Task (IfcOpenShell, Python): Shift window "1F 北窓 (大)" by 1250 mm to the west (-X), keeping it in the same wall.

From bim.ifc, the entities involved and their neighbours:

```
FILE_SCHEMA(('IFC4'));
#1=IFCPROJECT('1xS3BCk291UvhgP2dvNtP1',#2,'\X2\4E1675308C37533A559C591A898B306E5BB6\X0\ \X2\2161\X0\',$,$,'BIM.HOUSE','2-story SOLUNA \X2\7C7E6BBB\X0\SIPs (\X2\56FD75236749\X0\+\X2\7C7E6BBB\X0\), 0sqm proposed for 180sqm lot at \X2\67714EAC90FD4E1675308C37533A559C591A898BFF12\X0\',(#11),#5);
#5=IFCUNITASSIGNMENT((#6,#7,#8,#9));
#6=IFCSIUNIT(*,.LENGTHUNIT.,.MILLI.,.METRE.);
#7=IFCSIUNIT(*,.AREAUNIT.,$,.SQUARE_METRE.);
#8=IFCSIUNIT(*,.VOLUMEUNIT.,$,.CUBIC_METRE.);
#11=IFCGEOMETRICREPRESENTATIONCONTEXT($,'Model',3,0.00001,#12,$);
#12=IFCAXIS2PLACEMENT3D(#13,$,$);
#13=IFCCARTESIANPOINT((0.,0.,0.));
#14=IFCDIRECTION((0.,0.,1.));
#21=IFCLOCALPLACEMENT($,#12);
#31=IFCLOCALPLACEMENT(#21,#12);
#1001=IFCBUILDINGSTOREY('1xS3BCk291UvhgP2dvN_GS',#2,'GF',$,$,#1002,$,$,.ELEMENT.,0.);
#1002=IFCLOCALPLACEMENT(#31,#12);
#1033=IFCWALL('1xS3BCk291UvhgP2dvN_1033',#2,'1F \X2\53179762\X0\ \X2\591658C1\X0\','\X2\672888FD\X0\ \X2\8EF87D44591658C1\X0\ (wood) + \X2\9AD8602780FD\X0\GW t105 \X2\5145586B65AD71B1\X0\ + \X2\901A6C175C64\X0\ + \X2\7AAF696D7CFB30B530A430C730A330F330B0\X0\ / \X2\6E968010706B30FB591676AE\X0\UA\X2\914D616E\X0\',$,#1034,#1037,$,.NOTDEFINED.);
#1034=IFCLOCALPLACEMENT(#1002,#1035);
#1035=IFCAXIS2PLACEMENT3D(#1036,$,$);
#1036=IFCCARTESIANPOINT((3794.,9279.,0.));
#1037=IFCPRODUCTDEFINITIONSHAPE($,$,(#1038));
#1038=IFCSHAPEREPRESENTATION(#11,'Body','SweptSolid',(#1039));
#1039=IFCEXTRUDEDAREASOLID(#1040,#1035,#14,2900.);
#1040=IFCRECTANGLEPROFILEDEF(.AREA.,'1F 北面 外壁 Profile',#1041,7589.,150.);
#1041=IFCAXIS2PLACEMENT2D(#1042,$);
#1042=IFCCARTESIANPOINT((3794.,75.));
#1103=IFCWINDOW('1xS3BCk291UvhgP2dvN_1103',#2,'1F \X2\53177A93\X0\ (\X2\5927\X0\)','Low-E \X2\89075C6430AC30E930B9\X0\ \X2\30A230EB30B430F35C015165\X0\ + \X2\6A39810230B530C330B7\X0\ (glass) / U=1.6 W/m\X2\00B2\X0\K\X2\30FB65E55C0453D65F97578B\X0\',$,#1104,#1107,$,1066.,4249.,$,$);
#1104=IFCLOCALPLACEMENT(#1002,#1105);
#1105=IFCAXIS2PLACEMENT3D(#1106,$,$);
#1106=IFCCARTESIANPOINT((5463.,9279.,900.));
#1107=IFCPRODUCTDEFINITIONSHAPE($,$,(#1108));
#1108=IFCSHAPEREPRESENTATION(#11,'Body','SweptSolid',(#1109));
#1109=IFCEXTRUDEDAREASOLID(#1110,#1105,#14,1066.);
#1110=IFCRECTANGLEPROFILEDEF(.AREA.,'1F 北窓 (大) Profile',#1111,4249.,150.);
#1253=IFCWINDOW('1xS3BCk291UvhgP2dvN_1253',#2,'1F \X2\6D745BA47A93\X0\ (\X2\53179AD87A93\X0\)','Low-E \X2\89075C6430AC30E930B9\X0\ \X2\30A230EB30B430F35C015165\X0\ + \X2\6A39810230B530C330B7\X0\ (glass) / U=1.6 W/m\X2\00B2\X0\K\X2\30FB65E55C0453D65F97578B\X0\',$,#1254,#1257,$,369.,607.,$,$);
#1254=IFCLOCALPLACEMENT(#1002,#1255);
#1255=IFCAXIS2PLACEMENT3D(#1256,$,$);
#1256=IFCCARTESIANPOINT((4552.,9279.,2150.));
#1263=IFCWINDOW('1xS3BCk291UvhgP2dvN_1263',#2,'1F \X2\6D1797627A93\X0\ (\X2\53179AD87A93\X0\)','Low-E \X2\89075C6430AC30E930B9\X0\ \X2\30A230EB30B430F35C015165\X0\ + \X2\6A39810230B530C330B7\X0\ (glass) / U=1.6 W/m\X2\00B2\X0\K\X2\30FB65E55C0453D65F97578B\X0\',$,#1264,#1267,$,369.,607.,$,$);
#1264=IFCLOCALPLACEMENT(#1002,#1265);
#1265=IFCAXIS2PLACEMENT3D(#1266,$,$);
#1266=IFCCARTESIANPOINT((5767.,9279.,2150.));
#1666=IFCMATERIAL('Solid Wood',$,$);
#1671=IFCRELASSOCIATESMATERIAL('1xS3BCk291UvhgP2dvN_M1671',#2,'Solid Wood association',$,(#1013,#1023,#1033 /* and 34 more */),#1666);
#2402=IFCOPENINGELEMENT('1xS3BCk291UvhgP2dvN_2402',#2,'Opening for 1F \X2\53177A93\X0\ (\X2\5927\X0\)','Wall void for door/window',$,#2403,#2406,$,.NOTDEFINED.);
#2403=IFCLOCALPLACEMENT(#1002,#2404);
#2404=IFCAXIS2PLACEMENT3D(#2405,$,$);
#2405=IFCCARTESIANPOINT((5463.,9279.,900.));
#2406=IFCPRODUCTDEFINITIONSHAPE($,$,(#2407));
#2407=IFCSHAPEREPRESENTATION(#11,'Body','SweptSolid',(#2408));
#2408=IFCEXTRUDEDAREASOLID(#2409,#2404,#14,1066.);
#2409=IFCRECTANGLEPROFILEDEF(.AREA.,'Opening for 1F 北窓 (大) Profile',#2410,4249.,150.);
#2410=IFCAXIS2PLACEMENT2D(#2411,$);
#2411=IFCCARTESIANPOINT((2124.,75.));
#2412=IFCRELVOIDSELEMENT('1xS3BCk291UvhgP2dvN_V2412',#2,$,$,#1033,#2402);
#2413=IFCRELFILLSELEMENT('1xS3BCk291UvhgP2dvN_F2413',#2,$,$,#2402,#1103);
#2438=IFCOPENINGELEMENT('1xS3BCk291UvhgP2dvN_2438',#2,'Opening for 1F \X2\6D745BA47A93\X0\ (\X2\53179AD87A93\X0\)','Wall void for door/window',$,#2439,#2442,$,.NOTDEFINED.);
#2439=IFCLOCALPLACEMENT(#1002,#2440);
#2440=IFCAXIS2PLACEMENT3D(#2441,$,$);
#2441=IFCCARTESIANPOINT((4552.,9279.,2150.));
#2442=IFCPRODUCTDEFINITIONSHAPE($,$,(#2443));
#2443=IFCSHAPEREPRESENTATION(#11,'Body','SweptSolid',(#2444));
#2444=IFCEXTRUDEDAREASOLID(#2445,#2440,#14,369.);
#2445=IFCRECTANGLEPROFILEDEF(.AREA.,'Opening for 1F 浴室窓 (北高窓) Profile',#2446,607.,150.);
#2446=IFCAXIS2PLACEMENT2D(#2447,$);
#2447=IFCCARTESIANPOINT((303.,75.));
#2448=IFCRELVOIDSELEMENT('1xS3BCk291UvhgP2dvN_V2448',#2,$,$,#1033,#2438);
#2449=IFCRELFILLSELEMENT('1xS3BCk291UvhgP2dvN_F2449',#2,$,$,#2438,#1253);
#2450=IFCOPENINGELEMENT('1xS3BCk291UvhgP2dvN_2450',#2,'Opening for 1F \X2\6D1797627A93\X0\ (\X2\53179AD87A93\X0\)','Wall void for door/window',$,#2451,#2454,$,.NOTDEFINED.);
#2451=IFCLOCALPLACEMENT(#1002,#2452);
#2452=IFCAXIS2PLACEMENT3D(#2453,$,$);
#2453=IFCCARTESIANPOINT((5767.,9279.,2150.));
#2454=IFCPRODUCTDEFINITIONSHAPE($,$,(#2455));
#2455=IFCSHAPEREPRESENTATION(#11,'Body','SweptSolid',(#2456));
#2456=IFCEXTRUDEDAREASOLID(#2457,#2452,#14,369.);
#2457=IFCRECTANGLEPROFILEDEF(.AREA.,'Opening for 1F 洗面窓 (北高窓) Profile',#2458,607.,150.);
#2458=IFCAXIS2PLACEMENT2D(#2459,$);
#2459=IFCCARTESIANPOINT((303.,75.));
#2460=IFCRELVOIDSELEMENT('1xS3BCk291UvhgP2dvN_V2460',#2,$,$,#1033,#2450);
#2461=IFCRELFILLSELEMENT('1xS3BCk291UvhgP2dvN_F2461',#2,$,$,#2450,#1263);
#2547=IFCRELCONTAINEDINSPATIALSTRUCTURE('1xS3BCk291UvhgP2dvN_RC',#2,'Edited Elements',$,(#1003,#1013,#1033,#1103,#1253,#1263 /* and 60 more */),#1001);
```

```python
import ifcopenshell
import ifcopenshell.api.geometry
import ifcopenshell.util.placement
import ifcopenshell.util.unit

model = ifcopenshell.open("bim.ifc")
unit_scale = ifcopenshell.util.unit.calculate_unit_scale(model)

window = model.by_guid("1xS3BCk291UvhgP2dvN_1103")
opening = window.FillsVoids[0].RelatingOpeningElement
wall = opening.VoidsElements[0].RelatingBuildingElement

wall_matrix = ifcopenshell.util.placement.get_local_placement(wall.ObjectPlacement)
shift = wall_matrix[:3, 0] * -1.25 / unit_scale
before = ifcopenshell.util.placement.get_local_placement(window.ObjectPlacement)[:3, 3].copy()

# The window is not placed relative to its opening, so move both.
for product in (opening, window):
    matrix = ifcopenshell.util.placement.get_local_placement(product.ObjectPlacement)
    matrix[:3, 3] += shift
    ifcopenshell.api.geometry.edit_object_placement(model, product=product, matrix=matrix, is_si=False)

after = ifcopenshell.util.placement.get_local_placement(window.ObjectPlacement)[:3, 3]
print("window moved by", (after - before).round(3) + 0.0)

model.write("bim_v2.ifc")
```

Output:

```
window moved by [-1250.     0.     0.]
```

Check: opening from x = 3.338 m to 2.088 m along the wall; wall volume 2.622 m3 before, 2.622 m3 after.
